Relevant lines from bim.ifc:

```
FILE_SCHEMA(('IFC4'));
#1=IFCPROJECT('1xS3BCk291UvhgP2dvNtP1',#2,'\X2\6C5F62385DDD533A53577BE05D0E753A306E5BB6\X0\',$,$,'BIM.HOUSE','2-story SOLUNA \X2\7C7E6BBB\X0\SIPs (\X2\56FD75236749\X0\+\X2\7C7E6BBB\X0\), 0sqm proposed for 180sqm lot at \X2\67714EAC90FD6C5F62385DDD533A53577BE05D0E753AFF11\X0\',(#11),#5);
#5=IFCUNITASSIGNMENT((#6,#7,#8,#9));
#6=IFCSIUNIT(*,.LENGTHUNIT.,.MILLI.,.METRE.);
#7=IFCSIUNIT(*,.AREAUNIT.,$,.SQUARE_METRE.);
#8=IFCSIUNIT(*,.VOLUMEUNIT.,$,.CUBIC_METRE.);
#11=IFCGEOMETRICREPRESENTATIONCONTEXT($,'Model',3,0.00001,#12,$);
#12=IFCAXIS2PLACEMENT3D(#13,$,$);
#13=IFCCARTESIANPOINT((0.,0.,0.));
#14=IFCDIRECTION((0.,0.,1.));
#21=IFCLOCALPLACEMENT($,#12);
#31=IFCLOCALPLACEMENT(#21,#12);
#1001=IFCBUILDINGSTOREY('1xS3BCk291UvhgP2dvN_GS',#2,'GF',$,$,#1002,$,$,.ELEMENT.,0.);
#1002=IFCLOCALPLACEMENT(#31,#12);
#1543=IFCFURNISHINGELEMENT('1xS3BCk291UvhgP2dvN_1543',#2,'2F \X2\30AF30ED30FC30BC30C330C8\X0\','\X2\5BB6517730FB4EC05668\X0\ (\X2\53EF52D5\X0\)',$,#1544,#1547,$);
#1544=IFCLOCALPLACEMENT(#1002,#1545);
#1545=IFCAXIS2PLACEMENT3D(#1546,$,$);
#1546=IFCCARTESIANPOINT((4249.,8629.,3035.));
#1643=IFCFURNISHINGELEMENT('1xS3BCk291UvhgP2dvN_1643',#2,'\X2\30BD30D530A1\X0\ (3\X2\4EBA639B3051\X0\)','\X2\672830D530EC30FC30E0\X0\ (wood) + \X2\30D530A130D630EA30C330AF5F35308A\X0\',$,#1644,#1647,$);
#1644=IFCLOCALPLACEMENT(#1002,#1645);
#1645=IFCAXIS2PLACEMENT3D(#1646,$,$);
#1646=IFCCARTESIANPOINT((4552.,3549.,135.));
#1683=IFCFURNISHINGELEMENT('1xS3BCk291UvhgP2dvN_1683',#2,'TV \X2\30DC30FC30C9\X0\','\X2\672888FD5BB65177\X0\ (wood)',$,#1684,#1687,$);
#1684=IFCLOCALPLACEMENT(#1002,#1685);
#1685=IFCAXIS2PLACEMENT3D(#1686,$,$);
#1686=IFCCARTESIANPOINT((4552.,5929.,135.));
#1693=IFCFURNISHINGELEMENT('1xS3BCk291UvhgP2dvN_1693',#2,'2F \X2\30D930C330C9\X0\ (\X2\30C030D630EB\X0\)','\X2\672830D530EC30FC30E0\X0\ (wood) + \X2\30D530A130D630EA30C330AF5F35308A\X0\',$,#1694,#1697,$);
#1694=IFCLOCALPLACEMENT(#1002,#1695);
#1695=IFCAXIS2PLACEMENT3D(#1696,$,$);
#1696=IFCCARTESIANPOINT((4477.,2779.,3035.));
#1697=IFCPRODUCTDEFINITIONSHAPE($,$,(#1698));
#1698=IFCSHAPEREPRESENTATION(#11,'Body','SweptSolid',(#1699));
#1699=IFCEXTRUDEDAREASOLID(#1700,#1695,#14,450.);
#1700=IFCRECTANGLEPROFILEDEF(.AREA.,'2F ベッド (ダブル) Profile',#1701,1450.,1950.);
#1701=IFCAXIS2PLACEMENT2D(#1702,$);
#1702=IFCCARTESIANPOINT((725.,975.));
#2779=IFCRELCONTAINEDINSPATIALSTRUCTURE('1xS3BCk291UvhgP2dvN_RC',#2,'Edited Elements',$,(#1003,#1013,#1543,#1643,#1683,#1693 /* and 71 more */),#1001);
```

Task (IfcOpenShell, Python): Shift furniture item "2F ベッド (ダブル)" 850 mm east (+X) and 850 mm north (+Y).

```python
import ifcopenshell
import ifcopenshell.api.geometry
import ifcopenshell.util.placement
import ifcopenshell.util.unit

model = ifcopenshell.open("bim.ifc")
unit_scale = ifcopenshell.util.unit.calculate_unit_scale(model)

item = model.by_guid("1xS3BCk291UvhgP2dvN_1693")
matrix = ifcopenshell.util.placement.get_local_placement(item.ObjectPlacement)
matrix[0, 3] += 0.85 / unit_scale
matrix[1, 3] += 0.85 / unit_scale
ifcopenshell.api.geometry.edit_object_placement(model, product=item, matrix=matrix, is_si=False)

print(ifcopenshell.util.placement.get_local_placement(item.ObjectPlacement).round(3) + 0.0)

model.write("bim_v2.ifc")
```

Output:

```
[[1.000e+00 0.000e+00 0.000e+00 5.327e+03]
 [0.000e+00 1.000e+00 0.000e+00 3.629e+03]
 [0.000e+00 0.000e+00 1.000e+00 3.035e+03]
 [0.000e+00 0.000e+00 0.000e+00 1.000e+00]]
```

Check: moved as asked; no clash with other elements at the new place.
